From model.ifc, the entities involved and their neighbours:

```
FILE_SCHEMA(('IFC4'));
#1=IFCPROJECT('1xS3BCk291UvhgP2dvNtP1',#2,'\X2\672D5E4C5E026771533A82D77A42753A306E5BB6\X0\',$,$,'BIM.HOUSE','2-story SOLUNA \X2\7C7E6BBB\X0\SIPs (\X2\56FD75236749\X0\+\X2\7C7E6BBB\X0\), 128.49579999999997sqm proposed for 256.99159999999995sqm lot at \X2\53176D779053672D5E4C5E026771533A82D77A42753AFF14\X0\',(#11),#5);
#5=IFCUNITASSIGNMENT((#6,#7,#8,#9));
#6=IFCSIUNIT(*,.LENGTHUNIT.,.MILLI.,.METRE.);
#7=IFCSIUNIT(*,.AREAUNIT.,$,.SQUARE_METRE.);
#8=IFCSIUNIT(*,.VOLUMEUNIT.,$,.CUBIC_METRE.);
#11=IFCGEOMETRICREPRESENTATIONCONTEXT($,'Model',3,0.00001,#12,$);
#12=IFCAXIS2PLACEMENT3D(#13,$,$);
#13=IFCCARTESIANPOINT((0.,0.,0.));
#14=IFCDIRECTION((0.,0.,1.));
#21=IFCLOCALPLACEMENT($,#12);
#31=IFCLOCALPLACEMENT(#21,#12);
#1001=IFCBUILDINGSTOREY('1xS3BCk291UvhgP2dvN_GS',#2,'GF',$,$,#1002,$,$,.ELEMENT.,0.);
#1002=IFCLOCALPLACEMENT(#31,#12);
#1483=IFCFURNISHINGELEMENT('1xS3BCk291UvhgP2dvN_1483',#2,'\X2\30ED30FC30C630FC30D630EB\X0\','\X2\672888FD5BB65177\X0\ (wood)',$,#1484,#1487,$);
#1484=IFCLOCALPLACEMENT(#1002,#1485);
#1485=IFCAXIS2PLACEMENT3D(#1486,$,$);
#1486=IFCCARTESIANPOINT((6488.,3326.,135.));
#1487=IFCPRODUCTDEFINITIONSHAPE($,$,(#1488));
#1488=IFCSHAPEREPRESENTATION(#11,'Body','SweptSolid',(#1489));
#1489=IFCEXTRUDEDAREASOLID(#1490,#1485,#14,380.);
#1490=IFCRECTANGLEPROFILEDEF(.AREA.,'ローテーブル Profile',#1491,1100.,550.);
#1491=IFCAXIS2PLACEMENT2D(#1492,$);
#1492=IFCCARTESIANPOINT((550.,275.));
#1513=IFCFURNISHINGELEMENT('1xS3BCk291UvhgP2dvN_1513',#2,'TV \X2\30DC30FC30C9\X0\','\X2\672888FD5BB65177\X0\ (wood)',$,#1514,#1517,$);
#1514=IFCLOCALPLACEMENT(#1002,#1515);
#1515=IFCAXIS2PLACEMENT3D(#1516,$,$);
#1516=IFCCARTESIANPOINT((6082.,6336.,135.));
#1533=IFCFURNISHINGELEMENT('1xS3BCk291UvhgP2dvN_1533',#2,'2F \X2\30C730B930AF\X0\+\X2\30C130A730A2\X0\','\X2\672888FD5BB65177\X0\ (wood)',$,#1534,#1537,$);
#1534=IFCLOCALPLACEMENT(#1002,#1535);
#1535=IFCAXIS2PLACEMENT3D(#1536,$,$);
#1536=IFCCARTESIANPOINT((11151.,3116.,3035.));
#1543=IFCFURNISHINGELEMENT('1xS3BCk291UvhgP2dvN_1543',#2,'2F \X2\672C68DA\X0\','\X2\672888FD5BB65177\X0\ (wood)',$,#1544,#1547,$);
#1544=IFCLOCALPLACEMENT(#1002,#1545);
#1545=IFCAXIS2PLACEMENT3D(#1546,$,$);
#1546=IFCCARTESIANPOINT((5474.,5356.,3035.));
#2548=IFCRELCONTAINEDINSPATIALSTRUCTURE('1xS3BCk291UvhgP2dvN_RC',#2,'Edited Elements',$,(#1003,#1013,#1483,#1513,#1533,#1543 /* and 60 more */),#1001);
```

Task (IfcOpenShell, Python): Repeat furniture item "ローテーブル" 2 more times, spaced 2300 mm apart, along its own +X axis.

```python
import ifcopenshell
import ifcopenshell.api.geometry
import ifcopenshell.api.root
import ifcopenshell.util.element
import ifcopenshell.util.placement

model = ifcopenshell.open("model.ifc")


def reuse_history(source, copy):
    """copy_class also copies each property set's owner history, people and application; keep the originals."""
    for rel in copy.IsDefinedBy:
        if rel.is_a("IfcRelDefinesByProperties") and (history := rel.RelatingPropertyDefinition.OwnerHistory):
            rel.RelatingPropertyDefinition.OwnerHistory = source.OwnerHistory
            ifcopenshell.util.element.remove_deep2(model, history)


source = model.by_guid("1xS3BCk291UvhgP2dvN_1483")
base = ifcopenshell.util.placement.get_local_placement(source.ObjectPlacement)
step = base[:3, 0] * 2300.0

for i in range(1, 3):
    copy = ifcopenshell.api.root.copy_class(model, product=source)
    copy.Representation = ifcopenshell.util.element.copy_deep(
        model, source.Representation, exclude=["IfcGeometricRepresentationContext", "IfcRepresentationMap"]
    )
    reuse_history(source, copy)
    matrix = base.copy()
    matrix[:3, 3] += i * step
    print("added at", matrix[:3, 3].round(3) + 0.0)
    ifcopenshell.api.geometry.edit_object_placement(model, product=copy, matrix=matrix, is_si=False)

model.write("model_rev.ifc")
```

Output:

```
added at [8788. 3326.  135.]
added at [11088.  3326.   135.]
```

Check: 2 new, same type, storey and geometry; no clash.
